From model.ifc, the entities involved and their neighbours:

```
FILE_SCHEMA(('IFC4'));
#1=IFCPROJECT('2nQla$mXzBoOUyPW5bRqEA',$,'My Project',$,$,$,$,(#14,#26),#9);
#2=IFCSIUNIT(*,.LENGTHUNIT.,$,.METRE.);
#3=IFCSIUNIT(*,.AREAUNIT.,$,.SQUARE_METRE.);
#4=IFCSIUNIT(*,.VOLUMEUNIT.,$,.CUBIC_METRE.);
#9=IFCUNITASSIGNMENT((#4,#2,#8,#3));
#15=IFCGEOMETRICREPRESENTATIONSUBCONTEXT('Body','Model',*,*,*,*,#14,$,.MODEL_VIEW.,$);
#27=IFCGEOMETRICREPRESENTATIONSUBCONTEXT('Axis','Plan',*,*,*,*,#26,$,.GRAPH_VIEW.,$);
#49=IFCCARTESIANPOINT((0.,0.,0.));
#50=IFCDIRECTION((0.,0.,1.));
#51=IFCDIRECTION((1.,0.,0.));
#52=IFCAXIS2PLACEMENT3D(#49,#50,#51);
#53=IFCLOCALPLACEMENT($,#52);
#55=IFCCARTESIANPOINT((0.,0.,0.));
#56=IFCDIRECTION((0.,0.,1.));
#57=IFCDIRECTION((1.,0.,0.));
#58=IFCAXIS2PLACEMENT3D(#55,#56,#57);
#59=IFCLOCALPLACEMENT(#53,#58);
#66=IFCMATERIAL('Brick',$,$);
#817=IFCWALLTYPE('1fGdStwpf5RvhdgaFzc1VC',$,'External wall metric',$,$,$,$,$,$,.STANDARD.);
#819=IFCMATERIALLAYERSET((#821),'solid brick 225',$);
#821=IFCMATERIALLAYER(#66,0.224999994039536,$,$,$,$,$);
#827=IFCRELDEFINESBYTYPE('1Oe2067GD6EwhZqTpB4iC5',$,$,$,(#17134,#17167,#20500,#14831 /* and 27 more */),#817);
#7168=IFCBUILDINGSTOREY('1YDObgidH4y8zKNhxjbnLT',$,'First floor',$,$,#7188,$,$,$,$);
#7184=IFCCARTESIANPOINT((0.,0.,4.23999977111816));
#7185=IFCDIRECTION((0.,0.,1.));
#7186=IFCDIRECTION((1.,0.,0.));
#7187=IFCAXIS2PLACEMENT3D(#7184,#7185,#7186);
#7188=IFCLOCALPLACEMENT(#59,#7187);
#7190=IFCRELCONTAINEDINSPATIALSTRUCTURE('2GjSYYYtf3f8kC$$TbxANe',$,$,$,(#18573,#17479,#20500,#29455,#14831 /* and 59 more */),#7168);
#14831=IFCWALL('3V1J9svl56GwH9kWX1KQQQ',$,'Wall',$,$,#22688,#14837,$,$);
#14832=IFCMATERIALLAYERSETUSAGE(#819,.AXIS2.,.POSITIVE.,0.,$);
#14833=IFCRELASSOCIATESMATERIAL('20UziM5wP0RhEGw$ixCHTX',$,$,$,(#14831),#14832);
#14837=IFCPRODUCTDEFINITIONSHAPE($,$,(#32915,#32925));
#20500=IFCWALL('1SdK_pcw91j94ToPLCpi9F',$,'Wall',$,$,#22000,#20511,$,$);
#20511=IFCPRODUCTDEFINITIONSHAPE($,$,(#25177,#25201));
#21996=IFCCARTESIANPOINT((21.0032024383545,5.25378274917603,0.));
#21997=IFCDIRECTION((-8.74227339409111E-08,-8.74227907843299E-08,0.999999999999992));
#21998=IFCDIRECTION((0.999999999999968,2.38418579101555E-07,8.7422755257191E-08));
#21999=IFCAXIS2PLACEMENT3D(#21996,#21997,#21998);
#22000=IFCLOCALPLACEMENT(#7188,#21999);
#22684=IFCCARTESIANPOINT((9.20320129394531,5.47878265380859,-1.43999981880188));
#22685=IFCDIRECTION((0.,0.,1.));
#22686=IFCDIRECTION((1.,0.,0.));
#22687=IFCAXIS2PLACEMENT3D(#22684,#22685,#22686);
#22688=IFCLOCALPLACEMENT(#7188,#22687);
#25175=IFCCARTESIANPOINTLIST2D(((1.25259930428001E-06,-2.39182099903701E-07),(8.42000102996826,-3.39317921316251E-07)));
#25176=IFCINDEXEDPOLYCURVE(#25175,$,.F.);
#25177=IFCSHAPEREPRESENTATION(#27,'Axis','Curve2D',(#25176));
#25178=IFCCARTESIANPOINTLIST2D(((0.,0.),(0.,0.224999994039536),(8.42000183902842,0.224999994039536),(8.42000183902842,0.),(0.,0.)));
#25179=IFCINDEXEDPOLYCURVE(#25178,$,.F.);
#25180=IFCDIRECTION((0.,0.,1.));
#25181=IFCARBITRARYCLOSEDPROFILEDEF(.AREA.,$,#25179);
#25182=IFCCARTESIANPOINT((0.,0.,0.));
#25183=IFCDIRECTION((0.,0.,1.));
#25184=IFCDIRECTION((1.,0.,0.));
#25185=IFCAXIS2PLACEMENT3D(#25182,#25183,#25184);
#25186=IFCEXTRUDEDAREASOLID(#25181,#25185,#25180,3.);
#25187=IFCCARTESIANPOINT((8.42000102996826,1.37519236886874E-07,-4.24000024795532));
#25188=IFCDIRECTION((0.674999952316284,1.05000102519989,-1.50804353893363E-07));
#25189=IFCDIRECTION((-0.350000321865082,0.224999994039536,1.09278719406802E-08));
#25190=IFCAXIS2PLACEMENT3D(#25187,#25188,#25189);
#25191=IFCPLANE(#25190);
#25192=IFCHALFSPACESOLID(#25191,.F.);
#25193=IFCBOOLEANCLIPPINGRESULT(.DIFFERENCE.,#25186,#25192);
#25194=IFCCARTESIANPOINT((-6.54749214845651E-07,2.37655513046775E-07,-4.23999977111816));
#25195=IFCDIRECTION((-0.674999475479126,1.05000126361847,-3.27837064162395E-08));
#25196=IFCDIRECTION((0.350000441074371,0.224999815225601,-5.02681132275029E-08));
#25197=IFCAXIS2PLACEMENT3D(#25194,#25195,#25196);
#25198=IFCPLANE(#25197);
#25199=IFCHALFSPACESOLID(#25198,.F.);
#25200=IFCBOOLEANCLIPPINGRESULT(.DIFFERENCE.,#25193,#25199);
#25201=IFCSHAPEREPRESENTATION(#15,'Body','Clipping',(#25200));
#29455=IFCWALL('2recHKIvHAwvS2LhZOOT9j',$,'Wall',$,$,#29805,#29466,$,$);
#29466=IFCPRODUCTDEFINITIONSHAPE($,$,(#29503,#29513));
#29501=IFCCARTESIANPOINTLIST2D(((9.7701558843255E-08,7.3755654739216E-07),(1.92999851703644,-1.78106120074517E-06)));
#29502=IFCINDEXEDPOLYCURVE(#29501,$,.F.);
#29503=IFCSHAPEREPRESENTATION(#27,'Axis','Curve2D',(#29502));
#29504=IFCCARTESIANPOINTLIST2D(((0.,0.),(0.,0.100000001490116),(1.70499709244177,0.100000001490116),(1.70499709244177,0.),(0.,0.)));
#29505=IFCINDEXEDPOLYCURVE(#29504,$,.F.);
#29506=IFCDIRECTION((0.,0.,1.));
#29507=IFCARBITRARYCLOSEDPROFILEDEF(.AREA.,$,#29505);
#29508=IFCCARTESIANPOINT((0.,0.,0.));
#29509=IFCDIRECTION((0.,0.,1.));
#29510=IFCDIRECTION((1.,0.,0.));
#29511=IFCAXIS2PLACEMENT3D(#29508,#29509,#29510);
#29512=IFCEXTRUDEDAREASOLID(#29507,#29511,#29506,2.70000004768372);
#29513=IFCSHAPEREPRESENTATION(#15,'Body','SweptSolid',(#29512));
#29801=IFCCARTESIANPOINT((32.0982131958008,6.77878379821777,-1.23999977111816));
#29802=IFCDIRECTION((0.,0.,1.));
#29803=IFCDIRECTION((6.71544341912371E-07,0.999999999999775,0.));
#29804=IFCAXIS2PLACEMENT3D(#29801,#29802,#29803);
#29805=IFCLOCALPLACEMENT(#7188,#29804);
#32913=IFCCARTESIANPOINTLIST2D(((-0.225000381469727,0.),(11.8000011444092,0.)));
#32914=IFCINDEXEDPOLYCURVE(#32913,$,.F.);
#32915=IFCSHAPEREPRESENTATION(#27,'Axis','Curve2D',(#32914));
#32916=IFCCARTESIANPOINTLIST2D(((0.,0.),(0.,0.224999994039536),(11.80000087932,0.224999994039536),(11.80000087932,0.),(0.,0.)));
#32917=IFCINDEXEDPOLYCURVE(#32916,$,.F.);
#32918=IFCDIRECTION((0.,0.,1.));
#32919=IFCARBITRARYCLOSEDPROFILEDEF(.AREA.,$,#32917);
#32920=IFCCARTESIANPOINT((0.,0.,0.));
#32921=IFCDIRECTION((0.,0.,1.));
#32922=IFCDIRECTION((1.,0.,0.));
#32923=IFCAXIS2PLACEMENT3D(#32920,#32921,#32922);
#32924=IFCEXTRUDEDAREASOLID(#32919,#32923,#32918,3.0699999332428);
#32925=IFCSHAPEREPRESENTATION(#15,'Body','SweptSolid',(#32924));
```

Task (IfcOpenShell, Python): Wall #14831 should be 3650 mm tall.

```python
import ifcopenshell
import ifcopenshell.geom
import ifcopenshell.util.representation
import ifcopenshell.util.shape

model = ifcopenshell.open("model.ifc")
settings = ifcopenshell.geom.settings()


def volume(element):
    """Net volume in cubic metres, openings subtracted."""
    shape = ifcopenshell.geom.create_shape(settings, element)
    return ifcopenshell.util.shape.get_volume(shape.geometry)


wall = model.by_id(14831)
before = volume(wall)

body = ifcopenshell.util.representation.get_representation(wall, "Model", "Body")
solid = body.Items[0]
old_height = solid.Depth
solid.Depth = 3.65
after = volume(wall)

print(f"height {old_height:g} -> {solid.Depth:g}, volume {before:.3f} -> {after:.3f} m3")

model.write("model-out.ifc")
```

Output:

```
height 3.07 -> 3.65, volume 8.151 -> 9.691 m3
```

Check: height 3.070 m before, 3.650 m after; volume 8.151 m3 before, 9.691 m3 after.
